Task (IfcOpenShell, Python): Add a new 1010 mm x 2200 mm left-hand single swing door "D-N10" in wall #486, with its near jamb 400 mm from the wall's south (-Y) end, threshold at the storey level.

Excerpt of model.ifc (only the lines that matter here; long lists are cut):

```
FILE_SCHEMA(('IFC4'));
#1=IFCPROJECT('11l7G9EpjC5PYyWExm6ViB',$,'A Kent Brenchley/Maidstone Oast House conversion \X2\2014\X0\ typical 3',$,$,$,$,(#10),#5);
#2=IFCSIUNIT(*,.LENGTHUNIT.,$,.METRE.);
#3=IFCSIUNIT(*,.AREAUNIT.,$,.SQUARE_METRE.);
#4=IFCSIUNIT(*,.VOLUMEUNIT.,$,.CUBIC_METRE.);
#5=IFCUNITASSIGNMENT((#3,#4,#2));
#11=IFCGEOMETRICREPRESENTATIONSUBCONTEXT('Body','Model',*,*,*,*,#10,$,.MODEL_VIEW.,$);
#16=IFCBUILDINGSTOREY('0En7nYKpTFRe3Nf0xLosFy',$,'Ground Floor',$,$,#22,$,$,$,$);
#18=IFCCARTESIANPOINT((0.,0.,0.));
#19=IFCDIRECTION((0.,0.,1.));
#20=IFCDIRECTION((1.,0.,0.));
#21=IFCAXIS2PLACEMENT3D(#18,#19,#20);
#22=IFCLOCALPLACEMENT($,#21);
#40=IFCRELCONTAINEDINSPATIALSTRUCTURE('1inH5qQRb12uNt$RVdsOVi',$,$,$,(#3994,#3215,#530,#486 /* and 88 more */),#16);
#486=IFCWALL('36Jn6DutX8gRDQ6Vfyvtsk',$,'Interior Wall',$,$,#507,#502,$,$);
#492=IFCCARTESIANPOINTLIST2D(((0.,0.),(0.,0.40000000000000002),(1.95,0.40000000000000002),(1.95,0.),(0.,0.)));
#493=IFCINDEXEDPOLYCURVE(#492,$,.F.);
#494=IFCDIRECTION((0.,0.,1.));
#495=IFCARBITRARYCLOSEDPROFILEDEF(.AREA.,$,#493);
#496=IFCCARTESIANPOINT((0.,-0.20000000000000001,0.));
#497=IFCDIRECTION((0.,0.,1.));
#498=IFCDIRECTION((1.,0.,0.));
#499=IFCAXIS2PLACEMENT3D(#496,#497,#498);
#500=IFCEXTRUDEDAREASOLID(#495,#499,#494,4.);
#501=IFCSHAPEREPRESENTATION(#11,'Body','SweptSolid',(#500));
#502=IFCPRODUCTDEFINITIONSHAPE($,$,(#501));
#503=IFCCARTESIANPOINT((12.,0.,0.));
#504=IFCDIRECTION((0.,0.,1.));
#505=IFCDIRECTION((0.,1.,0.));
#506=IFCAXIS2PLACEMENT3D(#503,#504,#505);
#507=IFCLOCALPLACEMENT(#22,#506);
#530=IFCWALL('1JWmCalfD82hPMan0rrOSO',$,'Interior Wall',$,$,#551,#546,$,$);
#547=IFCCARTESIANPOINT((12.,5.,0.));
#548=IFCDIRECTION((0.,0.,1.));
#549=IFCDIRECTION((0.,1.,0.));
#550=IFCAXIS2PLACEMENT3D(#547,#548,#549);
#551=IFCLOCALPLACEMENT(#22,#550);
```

```python
import numpy as np
import ifcopenshell
import ifcopenshell.api.feature
import ifcopenshell.api.geometry
import ifcopenshell.api.root
import ifcopenshell.api.spatial
import ifcopenshell.geom
import ifcopenshell.util.element
import ifcopenshell.util.placement
import ifcopenshell.util.representation
import ifcopenshell.util.shape
import ifcopenshell.util.unit

model = ifcopenshell.open("model.ifc")
unit_scale = ifcopenshell.util.unit.calculate_unit_scale(model)
settings = ifcopenshell.geom.settings()


def volume(element):
    """Net volume in cubic metres, openings subtracted."""
    shape = ifcopenshell.geom.create_shape(settings, element)
    return ifcopenshell.util.shape.get_volume(shape.geometry)


wall = model.by_guid("36Jn6DutX8gRDQ6Vfyvtsk")
storey = ifcopenshell.util.element.get_container(wall, ifc_class="IfcBuildingStorey")
context = ifcopenshell.util.representation.get_context(model, "Model", "Body", "MODEL_VIEW")
before = volume(wall)

width, height, from_end, sill = 1.01, 2.2, 0.4, 0.0  # metres

# The wall runs along its own X axis, and the end named is its -X end.
wall_shape = ifcopenshell.geom.create_shape(settings, wall)
x, y, z = ifcopenshell.util.shape.get_vertices(wall_shape.geometry).T
start = x.min() + from_end
face, thickness = float(y.min()), float(y.max() - y.min())
wall_matrix = ifcopenshell.util.placement.get_local_placement(wall.ObjectPlacement)
level = ifcopenshell.util.placement.get_local_placement(storey.ObjectPlacement)[2, 3]


def in_wall(x, y):
    """Placement at x, y metres in the wall's axes, at sill height."""
    matrix = wall_matrix.copy()
    matrix[:, 3] = wall_matrix @ np.array([x / unit_scale, y / unit_scale, 0.0, 1.0])
    matrix[2, 3] = level + sill / unit_scale
    return matrix


# Opening: a box that overshoots both wall faces by 50 mm.
opening = ifcopenshell.api.root.create_entity(model, ifc_class="IfcOpeningElement", predefined_type="OPENING")
box = ifcopenshell.api.geometry.add_wall_representation(
    model, context=context, length=width, height=height, thickness=thickness + 0.1
)
ifcopenshell.api.geometry.assign_representation(model, product=opening, representation=box)
ifcopenshell.api.geometry.edit_object_placement(model, product=opening, matrix=in_wall(start, face - 0.05), is_si=False)
ifcopenshell.api.feature.add_feature(model, feature=opening, element=wall)

door = ifcopenshell.api.root.create_entity(model, ifc_class="IfcDoor", name="D-N10", predefined_type="DOOR")
door.OverallWidth, door.OverallHeight = width / unit_scale, height / unit_scale
door.OperationType = "SINGLE_SWING_LEFT"
body = ifcopenshell.api.geometry.add_door_representation(
    model,
    context=context,
    overall_width=door.OverallWidth,
    overall_height=door.OverallHeight,
    operation_type="SINGLE_SWING_LEFT",
    lining_properties={"LiningDepth": thickness / unit_scale, "ThresholdDepth": thickness / unit_scale},
)
ifcopenshell.api.geometry.assign_representation(model, product=door, representation=body)
ifcopenshell.api.spatial.assign_container(model, products=[door], relating_structure=storey)
ifcopenshell.api.feature.add_filling(model, opening=opening, element=door)

# The lining spans the wall, so the door starts at the wall face.
ifcopenshell.api.geometry.edit_object_placement(model, product=door, matrix=in_wall(start, face), is_si=False)

after = volume(wall)

print(f"wall volume {before:.3f} -> {after:.3f} m3")

model.write("model_rev.ifc")
```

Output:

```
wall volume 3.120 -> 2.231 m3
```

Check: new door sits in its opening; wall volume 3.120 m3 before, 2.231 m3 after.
